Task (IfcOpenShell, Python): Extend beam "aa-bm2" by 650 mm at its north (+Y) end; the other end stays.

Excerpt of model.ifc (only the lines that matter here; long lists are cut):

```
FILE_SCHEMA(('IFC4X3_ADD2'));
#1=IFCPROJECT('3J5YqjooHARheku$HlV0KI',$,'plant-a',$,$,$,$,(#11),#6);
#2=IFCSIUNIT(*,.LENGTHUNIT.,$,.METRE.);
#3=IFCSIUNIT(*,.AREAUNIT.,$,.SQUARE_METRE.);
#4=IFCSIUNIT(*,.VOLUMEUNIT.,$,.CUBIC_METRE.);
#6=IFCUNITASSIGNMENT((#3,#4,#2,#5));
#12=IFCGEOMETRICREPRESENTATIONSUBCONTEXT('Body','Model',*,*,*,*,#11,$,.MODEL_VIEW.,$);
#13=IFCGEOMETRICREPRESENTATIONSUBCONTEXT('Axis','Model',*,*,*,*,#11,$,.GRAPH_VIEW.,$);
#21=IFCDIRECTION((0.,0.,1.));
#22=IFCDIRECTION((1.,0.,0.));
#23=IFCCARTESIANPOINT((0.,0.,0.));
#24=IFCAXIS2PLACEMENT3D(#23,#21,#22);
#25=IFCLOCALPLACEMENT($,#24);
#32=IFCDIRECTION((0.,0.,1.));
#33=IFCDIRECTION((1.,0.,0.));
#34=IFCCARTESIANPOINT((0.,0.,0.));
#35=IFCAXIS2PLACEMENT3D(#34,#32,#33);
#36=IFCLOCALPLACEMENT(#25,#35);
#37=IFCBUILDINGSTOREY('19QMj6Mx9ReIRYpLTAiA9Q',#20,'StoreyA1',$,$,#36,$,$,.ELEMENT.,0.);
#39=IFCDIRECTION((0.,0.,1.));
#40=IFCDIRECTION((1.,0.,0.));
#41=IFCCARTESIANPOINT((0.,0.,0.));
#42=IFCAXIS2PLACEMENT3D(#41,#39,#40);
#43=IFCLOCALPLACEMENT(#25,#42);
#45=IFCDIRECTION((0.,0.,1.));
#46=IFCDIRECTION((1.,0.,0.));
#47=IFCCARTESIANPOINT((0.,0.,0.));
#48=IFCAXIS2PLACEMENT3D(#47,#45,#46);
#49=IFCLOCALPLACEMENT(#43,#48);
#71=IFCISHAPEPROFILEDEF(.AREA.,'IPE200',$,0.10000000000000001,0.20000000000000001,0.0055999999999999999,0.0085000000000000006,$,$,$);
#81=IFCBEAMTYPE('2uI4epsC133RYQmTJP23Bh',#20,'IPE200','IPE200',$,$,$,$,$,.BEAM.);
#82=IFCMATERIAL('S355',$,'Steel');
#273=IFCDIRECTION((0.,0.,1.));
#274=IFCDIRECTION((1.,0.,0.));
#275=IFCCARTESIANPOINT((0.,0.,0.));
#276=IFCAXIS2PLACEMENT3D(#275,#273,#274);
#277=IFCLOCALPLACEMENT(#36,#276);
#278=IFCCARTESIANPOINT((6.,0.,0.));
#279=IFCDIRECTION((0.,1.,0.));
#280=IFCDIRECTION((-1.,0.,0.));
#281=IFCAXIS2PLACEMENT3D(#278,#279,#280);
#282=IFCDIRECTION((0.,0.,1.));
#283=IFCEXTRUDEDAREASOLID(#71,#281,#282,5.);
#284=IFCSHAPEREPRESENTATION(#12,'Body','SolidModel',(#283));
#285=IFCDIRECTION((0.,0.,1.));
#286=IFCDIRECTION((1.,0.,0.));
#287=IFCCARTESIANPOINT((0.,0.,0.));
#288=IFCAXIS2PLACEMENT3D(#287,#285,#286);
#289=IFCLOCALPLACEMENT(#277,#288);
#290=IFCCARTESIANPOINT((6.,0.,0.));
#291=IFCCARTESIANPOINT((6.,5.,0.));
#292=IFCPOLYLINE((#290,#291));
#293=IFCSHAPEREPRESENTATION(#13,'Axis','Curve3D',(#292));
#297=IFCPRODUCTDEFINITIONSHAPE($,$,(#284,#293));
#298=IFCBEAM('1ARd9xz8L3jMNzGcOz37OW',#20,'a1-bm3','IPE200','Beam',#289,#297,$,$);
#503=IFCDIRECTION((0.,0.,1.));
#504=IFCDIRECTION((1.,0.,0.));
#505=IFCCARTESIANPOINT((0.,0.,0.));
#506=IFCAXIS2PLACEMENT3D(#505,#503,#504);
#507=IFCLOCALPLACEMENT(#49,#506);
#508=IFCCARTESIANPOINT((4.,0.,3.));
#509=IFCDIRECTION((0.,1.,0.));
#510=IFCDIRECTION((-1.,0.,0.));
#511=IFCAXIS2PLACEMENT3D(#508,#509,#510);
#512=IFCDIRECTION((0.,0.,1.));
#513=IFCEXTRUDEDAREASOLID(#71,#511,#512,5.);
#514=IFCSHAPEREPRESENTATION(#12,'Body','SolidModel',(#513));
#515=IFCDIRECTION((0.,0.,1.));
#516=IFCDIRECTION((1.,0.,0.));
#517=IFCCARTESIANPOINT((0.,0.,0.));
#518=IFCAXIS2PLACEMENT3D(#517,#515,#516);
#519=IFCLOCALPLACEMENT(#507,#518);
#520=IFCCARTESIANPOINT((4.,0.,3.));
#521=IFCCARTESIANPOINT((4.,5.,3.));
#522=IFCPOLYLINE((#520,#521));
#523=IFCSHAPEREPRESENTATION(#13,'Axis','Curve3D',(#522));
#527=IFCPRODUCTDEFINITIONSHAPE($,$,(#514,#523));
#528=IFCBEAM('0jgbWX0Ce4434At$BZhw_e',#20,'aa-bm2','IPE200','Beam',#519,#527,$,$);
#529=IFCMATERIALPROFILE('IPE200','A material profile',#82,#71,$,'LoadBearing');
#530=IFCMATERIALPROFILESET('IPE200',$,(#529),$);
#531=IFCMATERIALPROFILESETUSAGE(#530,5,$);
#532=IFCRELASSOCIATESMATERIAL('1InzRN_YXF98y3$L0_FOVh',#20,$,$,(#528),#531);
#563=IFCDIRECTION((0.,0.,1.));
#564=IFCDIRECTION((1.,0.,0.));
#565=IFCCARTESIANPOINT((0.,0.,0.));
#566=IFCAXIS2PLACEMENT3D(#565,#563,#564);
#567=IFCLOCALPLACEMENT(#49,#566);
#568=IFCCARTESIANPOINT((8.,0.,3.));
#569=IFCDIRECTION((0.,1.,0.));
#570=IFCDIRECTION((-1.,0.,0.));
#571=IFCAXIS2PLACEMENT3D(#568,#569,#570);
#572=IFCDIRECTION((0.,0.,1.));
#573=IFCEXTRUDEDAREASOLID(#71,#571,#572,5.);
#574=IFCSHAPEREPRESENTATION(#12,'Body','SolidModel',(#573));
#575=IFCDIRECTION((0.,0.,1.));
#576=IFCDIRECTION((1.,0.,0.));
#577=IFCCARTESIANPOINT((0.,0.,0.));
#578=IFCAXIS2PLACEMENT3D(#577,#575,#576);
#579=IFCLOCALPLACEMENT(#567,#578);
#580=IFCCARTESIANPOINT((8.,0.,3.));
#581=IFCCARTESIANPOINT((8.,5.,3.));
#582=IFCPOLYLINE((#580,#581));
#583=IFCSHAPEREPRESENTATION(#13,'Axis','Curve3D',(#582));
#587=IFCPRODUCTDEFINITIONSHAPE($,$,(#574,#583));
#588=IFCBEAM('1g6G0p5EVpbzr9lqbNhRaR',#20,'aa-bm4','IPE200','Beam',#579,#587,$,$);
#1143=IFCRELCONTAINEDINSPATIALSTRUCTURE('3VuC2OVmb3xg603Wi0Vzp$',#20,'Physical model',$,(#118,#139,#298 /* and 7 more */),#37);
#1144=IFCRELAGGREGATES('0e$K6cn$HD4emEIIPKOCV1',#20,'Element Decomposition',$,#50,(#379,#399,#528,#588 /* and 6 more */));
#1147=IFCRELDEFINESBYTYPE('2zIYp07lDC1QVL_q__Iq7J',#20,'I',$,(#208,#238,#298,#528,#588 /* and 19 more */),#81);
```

```python
import numpy as np
import ifcopenshell
import ifcopenshell.util.representation

model = ifcopenshell.open("model.ifc")

member = model.by_guid("0jgbWX0Ce4434At$BZhw_e")
change = 0.65

# The extrusion runs towards the end named, so only its depth changes.
body = ifcopenshell.util.representation.get_representation(member, "Model", "Body")
solid = body.Items[0]
old_length = solid.Depth
solid.Depth += change

# Move the axis end point with it.
axis = next(r for r in member.Representation.Representations if r.RepresentationIdentifier == "Axis").Items[0]
start, end = (np.array(p.Coordinates) for p in axis.Points)
end = end + (end - start) / np.linalg.norm(end - start) * change
point = model.createIfcCartesianPoint(end.tolist())
axis.Points = [axis.Points[0], point]

print(f"length {old_length:g} -> {solid.Depth:g}")

model.write("model_rev.ifc")
```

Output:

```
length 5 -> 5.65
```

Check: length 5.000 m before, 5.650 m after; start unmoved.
